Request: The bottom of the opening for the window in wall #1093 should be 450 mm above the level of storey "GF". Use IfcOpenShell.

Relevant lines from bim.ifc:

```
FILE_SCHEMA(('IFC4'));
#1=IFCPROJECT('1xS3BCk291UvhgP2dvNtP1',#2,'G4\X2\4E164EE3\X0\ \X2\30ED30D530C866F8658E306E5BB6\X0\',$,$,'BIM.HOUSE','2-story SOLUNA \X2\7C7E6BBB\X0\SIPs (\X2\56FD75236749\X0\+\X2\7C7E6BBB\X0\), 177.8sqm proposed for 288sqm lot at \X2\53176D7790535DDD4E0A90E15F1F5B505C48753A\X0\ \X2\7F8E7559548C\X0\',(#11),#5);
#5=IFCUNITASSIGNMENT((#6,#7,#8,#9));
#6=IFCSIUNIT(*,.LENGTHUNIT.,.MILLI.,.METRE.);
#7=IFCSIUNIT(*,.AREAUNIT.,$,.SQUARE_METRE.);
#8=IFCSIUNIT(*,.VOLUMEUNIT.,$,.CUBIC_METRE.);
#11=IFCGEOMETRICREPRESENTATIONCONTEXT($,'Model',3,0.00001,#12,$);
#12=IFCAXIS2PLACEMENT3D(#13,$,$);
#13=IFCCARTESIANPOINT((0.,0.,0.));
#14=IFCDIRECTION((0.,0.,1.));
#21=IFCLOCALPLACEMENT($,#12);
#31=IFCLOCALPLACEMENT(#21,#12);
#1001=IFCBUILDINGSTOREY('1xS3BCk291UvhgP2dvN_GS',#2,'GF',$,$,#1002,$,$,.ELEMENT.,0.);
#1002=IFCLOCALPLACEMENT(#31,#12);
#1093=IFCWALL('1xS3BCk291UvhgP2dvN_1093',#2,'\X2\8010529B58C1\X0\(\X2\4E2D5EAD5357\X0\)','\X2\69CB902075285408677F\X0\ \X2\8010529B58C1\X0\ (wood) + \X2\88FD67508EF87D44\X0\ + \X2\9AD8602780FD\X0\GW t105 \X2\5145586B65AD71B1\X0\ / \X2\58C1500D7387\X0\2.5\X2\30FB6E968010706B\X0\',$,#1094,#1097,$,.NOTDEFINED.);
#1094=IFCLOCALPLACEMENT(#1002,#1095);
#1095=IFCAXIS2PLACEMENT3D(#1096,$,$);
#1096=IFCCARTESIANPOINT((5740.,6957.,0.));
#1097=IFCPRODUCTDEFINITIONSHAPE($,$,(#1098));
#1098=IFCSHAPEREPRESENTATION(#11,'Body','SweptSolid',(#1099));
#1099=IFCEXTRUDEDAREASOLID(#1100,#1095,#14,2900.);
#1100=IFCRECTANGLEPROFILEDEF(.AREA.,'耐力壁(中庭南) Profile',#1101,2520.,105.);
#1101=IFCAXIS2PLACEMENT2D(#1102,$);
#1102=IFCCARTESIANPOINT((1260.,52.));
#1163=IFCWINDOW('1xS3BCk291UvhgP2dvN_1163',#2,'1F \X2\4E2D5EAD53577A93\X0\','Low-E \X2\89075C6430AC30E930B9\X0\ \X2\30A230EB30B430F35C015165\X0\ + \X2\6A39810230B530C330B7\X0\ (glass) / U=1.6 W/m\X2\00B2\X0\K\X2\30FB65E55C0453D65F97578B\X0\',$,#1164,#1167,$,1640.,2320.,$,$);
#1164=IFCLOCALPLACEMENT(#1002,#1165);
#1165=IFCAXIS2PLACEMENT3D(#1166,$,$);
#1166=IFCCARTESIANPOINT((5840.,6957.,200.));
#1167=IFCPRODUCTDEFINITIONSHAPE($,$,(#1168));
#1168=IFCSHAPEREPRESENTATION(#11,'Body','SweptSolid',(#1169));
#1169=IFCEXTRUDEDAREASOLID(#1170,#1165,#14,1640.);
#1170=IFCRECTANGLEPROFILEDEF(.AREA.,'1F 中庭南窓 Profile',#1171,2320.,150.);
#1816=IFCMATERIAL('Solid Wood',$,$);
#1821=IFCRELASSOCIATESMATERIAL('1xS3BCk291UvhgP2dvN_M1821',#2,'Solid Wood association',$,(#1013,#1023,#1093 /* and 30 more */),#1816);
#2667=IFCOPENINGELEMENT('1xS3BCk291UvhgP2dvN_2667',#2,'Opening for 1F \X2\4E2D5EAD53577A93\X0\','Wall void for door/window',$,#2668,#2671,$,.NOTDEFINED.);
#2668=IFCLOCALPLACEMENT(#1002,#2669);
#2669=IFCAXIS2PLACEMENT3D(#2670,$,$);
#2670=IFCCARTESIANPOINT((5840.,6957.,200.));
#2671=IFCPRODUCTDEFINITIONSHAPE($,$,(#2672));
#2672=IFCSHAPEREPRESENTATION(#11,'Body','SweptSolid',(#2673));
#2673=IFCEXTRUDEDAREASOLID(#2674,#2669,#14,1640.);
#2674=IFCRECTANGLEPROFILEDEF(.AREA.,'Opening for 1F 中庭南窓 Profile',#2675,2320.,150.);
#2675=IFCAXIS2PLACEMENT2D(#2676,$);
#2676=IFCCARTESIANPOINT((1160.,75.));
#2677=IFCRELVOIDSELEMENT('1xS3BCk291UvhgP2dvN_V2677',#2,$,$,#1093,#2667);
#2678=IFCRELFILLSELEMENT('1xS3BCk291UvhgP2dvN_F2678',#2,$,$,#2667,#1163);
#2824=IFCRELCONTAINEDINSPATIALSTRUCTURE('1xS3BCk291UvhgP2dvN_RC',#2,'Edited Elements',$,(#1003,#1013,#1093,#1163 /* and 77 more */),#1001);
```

```python
import numpy as np
import ifcopenshell
import ifcopenshell.api.geometry
import ifcopenshell.geom
import ifcopenshell.util.element
import ifcopenshell.util.placement
import ifcopenshell.util.shape
import ifcopenshell.util.unit

model = ifcopenshell.open("bim.ifc")
unit_scale = ifcopenshell.util.unit.calculate_unit_scale(model)

window = model.by_guid("1xS3BCk291UvhgP2dvN_1163")
opening = window.FillsVoids[0].RelatingOpeningElement
storey = ifcopenshell.util.element.get_container(window, ifc_class="IfcBuildingStorey")
level = ifcopenshell.util.placement.get_local_placement(storey.ObjectPlacement)[2, 3]

# The opening's origin need not be at the sill, so measure its lowest point.
shape = ifcopenshell.geom.create_shape(ifcopenshell.geom.settings(), opening)
bottom = ifcopenshell.util.shape.get_shape_bottom_elevation(shape, shape.geometry) / unit_scale
dz = level + 0.45 / unit_scale - bottom

shift = np.array([0.0, 0.0, dz])
# The window is not placed relative to its opening, so move both.
for product in (opening, window):
    matrix = ifcopenshell.util.placement.get_local_placement(product.ObjectPlacement)
    matrix[:3, 3] += shift
    ifcopenshell.api.geometry.edit_object_placement(model, product=product, matrix=matrix, is_si=False)

print(f"moved by {dz * unit_scale:+.3f} m")

model.write("bim_rev.ifc")
```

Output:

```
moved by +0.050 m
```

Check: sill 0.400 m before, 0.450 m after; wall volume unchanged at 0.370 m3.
